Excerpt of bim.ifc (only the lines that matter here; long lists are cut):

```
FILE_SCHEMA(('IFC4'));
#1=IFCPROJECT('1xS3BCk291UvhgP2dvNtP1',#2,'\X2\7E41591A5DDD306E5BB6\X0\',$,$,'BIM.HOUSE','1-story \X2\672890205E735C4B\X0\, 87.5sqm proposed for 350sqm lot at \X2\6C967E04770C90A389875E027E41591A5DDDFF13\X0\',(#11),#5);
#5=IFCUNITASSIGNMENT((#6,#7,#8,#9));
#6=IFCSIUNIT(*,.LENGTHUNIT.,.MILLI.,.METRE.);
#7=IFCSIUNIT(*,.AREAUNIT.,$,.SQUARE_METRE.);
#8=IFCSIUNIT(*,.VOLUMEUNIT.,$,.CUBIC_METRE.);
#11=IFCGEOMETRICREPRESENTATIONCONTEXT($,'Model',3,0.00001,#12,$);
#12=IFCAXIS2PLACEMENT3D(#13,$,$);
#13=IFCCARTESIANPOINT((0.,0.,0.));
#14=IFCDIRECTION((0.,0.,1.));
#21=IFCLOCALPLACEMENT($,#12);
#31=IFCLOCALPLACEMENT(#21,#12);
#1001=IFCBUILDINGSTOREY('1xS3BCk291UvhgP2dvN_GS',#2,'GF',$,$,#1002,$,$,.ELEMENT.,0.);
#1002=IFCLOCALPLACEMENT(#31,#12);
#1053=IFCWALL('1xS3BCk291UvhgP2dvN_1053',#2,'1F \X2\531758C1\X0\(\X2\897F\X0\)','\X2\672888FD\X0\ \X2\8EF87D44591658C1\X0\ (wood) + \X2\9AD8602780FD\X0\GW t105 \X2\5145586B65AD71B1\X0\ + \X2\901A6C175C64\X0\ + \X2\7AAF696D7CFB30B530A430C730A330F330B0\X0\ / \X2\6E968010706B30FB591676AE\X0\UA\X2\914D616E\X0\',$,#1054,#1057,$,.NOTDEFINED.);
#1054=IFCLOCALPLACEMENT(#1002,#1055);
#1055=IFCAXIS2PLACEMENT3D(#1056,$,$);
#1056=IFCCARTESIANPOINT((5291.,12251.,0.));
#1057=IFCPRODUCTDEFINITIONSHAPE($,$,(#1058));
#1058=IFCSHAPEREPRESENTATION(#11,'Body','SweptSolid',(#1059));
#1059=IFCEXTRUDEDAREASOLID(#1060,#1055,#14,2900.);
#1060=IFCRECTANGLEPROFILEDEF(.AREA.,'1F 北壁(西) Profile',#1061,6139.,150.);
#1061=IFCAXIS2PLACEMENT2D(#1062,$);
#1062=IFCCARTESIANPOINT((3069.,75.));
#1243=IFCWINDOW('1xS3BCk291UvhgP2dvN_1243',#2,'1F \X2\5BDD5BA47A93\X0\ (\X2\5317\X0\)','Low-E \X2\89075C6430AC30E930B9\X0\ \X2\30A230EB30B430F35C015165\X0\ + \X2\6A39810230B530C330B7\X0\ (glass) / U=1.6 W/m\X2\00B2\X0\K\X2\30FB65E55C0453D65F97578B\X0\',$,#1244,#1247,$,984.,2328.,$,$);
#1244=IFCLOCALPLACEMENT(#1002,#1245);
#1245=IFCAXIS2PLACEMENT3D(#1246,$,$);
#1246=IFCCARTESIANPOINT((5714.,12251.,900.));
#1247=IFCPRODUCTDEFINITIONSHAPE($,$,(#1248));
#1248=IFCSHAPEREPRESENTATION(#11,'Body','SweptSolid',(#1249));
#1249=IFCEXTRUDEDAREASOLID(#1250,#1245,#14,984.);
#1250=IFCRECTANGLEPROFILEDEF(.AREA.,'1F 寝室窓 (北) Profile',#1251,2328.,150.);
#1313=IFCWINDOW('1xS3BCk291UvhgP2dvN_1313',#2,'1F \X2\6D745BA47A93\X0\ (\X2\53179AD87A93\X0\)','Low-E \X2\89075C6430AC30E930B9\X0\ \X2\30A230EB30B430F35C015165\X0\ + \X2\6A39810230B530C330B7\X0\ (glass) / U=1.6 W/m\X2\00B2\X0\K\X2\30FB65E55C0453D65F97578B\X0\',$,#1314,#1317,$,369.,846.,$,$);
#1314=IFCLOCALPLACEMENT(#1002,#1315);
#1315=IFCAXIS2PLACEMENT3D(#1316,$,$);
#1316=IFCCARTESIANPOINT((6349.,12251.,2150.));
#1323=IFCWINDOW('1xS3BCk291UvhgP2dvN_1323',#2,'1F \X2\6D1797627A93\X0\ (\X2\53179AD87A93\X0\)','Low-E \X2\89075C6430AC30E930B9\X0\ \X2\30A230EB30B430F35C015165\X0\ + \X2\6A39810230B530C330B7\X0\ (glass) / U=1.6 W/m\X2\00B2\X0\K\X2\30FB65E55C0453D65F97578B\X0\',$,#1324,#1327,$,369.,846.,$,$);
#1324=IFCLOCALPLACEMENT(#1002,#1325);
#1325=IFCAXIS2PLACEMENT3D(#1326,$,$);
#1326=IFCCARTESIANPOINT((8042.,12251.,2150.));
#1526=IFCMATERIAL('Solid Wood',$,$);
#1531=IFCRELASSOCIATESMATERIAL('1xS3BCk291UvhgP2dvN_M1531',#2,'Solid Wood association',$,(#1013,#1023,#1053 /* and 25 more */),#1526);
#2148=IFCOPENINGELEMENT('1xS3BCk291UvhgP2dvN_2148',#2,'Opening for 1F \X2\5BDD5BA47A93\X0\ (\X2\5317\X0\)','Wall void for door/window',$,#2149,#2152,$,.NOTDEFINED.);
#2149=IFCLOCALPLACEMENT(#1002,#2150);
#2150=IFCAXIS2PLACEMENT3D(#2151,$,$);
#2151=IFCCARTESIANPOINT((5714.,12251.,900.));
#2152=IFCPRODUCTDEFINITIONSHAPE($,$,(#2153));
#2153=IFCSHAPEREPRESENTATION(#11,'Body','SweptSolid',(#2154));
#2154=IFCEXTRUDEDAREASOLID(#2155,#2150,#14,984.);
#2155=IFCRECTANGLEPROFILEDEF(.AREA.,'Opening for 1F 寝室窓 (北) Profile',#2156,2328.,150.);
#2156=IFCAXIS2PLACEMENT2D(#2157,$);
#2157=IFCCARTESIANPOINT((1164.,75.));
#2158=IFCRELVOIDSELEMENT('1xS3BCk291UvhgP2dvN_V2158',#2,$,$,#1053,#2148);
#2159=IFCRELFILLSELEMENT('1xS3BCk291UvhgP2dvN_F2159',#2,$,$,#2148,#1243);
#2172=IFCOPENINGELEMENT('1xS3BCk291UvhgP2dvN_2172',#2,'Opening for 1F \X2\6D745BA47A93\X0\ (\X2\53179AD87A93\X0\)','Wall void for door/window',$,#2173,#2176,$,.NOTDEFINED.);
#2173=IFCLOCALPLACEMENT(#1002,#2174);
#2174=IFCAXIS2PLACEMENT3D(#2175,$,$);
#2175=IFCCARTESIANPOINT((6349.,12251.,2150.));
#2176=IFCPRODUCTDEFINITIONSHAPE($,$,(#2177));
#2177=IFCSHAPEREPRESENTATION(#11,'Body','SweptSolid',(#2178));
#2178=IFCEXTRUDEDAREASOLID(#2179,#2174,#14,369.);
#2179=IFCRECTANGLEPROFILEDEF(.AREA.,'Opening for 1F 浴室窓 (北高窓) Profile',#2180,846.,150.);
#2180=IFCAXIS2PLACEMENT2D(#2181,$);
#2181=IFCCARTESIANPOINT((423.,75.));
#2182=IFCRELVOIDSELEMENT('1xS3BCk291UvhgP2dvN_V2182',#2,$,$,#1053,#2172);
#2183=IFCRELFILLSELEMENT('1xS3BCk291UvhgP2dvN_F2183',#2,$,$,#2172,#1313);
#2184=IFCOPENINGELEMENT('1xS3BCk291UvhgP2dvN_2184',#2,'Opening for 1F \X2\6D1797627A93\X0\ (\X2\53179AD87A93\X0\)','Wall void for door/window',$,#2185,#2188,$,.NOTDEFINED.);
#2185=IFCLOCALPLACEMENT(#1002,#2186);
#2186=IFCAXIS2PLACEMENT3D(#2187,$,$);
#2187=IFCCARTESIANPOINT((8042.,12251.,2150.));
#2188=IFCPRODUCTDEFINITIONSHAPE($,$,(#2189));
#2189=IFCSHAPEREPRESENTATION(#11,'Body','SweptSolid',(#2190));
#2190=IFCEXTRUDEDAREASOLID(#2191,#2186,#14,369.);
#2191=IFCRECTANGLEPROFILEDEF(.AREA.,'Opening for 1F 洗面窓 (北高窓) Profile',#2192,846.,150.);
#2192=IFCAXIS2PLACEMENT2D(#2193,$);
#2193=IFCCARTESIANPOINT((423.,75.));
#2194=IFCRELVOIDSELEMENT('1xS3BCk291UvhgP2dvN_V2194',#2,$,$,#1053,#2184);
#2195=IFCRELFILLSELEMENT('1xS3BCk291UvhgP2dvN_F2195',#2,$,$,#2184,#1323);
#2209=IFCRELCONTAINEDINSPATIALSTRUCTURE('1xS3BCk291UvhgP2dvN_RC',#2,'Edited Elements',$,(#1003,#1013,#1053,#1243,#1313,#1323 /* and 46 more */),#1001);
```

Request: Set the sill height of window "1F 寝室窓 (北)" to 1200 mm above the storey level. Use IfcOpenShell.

```python
import numpy as np
import ifcopenshell
import ifcopenshell.api.geometry
import ifcopenshell.geom
import ifcopenshell.util.element
import ifcopenshell.util.placement
import ifcopenshell.util.shape
import ifcopenshell.util.unit

model = ifcopenshell.open("bim.ifc")
unit_scale = ifcopenshell.util.unit.calculate_unit_scale(model)

window = model.by_guid("1xS3BCk291UvhgP2dvN_1243")
opening = window.FillsVoids[0].RelatingOpeningElement
storey = ifcopenshell.util.element.get_container(window, ifc_class="IfcBuildingStorey")
level = ifcopenshell.util.placement.get_local_placement(storey.ObjectPlacement)[2, 3]

# The opening's origin need not be at the sill, so measure its lowest point.
shape = ifcopenshell.geom.create_shape(ifcopenshell.geom.settings(), opening)
bottom = ifcopenshell.util.shape.get_shape_bottom_elevation(shape, shape.geometry) / unit_scale
dz = level + 1.2 / unit_scale - bottom

shift = np.array([0.0, 0.0, dz])
# The window is not placed relative to its opening, so move both.
for product in (opening, window):
    matrix = ifcopenshell.util.placement.get_local_placement(product.ObjectPlacement)
    matrix[:3, 3] += shift
    ifcopenshell.api.geometry.edit_object_placement(model, product=product, matrix=matrix, is_si=False)

print(f"moved by {dz * unit_scale:+.3f} m")

model.write("bim-out.ifc")
```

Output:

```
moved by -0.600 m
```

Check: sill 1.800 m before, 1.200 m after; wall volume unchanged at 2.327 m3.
